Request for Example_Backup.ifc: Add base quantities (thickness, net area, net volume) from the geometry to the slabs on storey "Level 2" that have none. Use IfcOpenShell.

First a look at what the model holds.

```python
import ifcopenshell
import ifcopenshell.util.element
import ifcopenshell.util.unit

model = ifcopenshell.open("Example_Backup.ifc")
print(model.schema)
for unit_type in ("LENGTHUNIT", "AREAUNIT", "VOLUMEUNIT"):
    print(unit_type, ifcopenshell.util.unit.calculate_unit_scale(model, unit_type))
storey = next(s for s in model.by_type("IfcBuildingStorey") if s.Name == "Level 2")
slabs = [e for e in ifcopenshell.util.element.get_decomposition(storey) if e.is_a("IfcSlab")]
for e in sorted(slabs, key=lambda e: e.id()):
    print(e.id(), e.is_a(), e.Name, list(ifcopenshell.util.element.get_psets(e, qtos_only=True)), sep=" | ")
```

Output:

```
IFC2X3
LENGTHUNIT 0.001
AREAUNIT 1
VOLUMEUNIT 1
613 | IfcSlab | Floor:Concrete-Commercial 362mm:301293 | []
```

```python
import ifcopenshell
import ifcopenshell.api.pset
import ifcopenshell.geom
import ifcopenshell.util.element
import ifcopenshell.util.shape
import ifcopenshell.util.unit

model = ifcopenshell.open("Example_Backup.ifc")
unit_scale = ifcopenshell.util.unit.calculate_unit_scale(model)
area_scale = ifcopenshell.util.unit.calculate_unit_scale(model, "AREAUNIT")
volume_scale = ifcopenshell.util.unit.calculate_unit_scale(model, "VOLUMEUNIT")
settings = ifcopenshell.geom.settings()

storey = next(s for s in model.by_type("IfcBuildingStorey") if s.Name == "Level 2")
slabs = [e for e in ifcopenshell.util.element.get_decomposition(storey) if e.is_a("IfcSlab")]

for e in sorted(slabs, key=lambda e: e.id()):
    if ifcopenshell.util.element.get_psets(e, qtos_only=True, should_inherit=False):
        continue
    # Geometry comes back in metres, in the element's own axes.
    shape = ifcopenshell.geom.create_shape(settings, e)
    values = {
        "Width": ifcopenshell.util.shape.get_z(shape.geometry) / unit_scale,
        "NetArea": ifcopenshell.util.shape.get_footprint_area(shape.geometry) / area_scale,
        "NetVolume": ifcopenshell.util.shape.get_volume(shape.geometry) / volume_scale,
    }
    qto = ifcopenshell.api.pset.add_qto(model, product=e, name="BaseQuantities")
    ifcopenshell.api.pset.edit_qto(model, qto=qto, properties=values)
    print(e.id(), {k: round(v, 3) for k, v in values.items()})

model.write("Example_Backup_edited.ifc")
```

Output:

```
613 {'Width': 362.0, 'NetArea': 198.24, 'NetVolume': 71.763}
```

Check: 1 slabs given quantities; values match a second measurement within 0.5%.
